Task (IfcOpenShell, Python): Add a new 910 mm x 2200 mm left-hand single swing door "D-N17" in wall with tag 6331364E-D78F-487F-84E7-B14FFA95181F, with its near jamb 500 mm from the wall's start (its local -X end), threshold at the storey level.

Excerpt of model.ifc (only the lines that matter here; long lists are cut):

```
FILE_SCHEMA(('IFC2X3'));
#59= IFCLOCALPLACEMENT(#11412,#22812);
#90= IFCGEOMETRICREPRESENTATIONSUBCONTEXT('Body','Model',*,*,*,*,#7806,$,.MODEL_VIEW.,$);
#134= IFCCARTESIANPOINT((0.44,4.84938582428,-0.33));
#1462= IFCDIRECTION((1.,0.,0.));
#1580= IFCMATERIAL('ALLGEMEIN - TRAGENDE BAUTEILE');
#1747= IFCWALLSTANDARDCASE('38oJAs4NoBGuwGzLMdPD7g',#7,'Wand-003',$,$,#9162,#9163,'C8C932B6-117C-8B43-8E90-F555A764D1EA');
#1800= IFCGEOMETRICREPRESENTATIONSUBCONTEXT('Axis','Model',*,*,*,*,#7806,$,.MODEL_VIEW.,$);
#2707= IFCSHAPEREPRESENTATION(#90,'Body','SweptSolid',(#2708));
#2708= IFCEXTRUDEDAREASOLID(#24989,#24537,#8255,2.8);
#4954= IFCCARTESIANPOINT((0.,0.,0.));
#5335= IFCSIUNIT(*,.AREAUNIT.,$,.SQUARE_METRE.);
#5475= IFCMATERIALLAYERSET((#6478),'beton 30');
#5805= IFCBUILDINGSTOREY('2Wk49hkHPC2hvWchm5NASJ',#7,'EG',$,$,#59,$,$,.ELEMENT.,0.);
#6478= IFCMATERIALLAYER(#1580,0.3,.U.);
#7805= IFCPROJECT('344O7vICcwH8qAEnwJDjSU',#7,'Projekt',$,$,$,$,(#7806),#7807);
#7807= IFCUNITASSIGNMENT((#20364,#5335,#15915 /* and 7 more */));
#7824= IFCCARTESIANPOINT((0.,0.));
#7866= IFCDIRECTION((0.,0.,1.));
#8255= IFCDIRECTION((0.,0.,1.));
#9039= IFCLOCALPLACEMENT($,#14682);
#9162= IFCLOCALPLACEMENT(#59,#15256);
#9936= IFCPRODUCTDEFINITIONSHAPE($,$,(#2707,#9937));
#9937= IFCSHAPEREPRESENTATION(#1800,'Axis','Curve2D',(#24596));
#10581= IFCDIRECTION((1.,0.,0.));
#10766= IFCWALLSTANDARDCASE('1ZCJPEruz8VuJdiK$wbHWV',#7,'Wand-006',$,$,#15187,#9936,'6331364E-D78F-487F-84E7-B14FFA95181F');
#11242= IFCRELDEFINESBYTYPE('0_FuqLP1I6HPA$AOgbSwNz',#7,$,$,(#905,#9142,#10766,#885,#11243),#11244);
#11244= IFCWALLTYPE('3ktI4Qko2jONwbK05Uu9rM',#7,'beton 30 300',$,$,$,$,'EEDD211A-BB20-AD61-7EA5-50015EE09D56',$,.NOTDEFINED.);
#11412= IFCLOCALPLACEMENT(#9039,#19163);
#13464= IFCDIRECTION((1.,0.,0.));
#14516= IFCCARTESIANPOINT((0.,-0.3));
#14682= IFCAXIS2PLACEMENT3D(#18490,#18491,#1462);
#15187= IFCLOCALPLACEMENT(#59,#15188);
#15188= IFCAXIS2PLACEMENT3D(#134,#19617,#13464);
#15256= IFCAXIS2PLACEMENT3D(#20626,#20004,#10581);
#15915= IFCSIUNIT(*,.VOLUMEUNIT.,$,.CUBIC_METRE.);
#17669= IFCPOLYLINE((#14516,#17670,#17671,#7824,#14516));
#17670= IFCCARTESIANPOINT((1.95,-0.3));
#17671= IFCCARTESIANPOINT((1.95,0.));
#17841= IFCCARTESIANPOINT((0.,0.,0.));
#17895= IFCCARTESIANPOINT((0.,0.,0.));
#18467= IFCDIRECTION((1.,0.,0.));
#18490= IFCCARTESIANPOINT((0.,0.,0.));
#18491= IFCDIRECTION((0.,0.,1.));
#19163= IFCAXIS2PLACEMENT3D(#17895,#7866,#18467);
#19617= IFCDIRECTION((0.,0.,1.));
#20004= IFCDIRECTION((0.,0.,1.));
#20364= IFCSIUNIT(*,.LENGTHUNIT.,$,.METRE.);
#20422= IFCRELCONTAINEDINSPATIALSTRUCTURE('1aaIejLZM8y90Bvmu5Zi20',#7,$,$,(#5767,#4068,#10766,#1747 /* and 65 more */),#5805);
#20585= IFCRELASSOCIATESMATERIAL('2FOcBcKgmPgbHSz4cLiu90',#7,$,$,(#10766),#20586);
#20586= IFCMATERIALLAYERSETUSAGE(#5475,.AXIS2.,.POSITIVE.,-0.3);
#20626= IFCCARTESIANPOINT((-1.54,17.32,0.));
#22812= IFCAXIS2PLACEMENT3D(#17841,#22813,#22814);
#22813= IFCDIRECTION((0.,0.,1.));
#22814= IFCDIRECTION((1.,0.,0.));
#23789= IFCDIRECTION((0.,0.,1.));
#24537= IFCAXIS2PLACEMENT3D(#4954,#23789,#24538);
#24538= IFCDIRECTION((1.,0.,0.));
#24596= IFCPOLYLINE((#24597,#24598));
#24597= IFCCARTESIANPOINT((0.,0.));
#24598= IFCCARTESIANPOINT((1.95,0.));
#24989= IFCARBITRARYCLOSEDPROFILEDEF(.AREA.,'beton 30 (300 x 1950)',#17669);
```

```python
import numpy as np
import ifcopenshell
import ifcopenshell.api.feature
import ifcopenshell.api.geometry
import ifcopenshell.api.root
import ifcopenshell.api.spatial
import ifcopenshell.api.type
import ifcopenshell.geom
import ifcopenshell.util.element
import ifcopenshell.util.placement
import ifcopenshell.util.representation
import ifcopenshell.util.shape
import ifcopenshell.util.unit

model = ifcopenshell.open("model.ifc")
unit_scale = ifcopenshell.util.unit.calculate_unit_scale(model)
settings = ifcopenshell.geom.settings()


def volume(element):
    """Net volume in cubic metres, openings subtracted."""
    shape = ifcopenshell.geom.create_shape(settings, element)
    return ifcopenshell.util.shape.get_volume(shape.geometry)


wall = model.by_guid("1ZCJPEruz8VuJdiK$wbHWV")
storey = ifcopenshell.util.element.get_container(wall, ifc_class="IfcBuildingStorey")
context = ifcopenshell.util.representation.get_context(model, "Model", "Body", "MODEL_VIEW")
before = volume(wall)

width, height, from_end, sill = 0.91, 2.2, 0.5, 0.0  # metres

# The wall runs along its own X axis, and the end named is its -X end.
wall_shape = ifcopenshell.geom.create_shape(settings, wall)
x, y, z = ifcopenshell.util.shape.get_vertices(wall_shape.geometry).T
start = x.min() + from_end
face, thickness = float(y.min()), float(y.max() - y.min())
wall_matrix = ifcopenshell.util.placement.get_local_placement(wall.ObjectPlacement)
level = ifcopenshell.util.placement.get_local_placement(storey.ObjectPlacement)[2, 3]


def in_wall(x, y):
    """Placement at x, y metres in the wall's axes, at sill height."""
    matrix = wall_matrix.copy()
    matrix[:, 3] = wall_matrix @ np.array([x / unit_scale, y / unit_scale, 0.0, 1.0])
    matrix[2, 3] = level + sill / unit_scale
    return matrix


# Opening: a box that overshoots both wall faces by 50 mm.
opening = ifcopenshell.api.root.create_entity(model, ifc_class="IfcOpeningElement")
box = ifcopenshell.api.geometry.add_wall_representation(
    model, context=context, length=width, height=height, thickness=thickness + 0.1
)
ifcopenshell.api.geometry.assign_representation(model, product=opening, representation=box)
ifcopenshell.api.geometry.edit_object_placement(model, product=opening, matrix=in_wall(start, face - 0.05), is_si=False)
ifcopenshell.api.feature.add_feature(model, feature=opening, element=wall)

door = ifcopenshell.api.root.create_entity(model, ifc_class="IfcDoor", name="D-N17")
door.OverallWidth, door.OverallHeight = width / unit_scale, height / unit_scale
body = ifcopenshell.api.geometry.add_door_representation(
    model,
    context=context,
    overall_width=door.OverallWidth,
    overall_height=door.OverallHeight,
    operation_type="SINGLE_SWING_LEFT",
    lining_properties={"LiningDepth": thickness / unit_scale, "ThresholdDepth": thickness / unit_scale},
)
ifcopenshell.api.geometry.assign_representation(model, product=door, representation=body)
ifcopenshell.api.spatial.assign_container(model, products=[door], relating_structure=storey)
fills = ifcopenshell.api.feature.add_filling(model, opening=opening, element=door)
fills.OwnerHistory = door.OwnerHistory  # required in IFC2X3

# IFC2X3 keeps the operation on the door style.
style = ifcopenshell.api.root.create_entity(model, ifc_class="IfcDoorStyle", name="D-N17")
style.OperationType, style.ConstructionType = "SINGLE_SWING_LEFT", "NOTDEFINED"
style.ParameterTakesPrecedence = style.Sizeable = False
ifcopenshell.api.type.assign_type(model, related_objects=[door], relating_type=style)

# The lining spans the wall, so the door starts at the wall face.
ifcopenshell.api.geometry.edit_object_placement(model, product=door, matrix=in_wall(start, face), is_si=False)

after = volume(wall)

print(f"wall volume {before:.3f} -> {after:.3f} m3")

model.write("model_v2.ifc")
```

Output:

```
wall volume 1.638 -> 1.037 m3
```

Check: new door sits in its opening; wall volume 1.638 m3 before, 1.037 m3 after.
